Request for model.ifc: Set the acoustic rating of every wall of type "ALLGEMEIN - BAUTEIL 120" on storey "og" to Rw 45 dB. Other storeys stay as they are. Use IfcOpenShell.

First a look at what the model holds.

```python
import ifcopenshell
import ifcopenshell.util.element

model = ifcopenshell.open("model.ifc")
print(model.schema)
storey = next(s for s in model.by_type("IfcBuildingStorey") if s.Name == "og")
walls = [e for e in ifcopenshell.util.element.get_decomposition(storey) if e.is_a("IfcWall")]
seen = {}
for e in walls:
    element_type = ifcopenshell.util.element.get_type(e)
    key = (element_type.Name if element_type != e and element_type else None, ifcopenshell.util.element.get_pset(e, "Pset_WallCommon", "AcousticRating"))
    seen[key] = seen.get(key, 0) + 1
for (name, value), count in sorted(seen.items(), key=str):
    print(count, "x", name, "|", value)
```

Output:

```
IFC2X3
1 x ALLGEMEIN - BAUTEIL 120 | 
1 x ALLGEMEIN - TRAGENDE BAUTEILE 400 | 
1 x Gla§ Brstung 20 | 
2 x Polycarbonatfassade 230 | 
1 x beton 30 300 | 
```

```python
import ifcopenshell
import ifcopenshell.api.pset
import ifcopenshell.util.element

model = ifcopenshell.open("model.ifc")

storey = next(s for s in model.by_type("IfcBuildingStorey") if s.Name == "og")
walls = [e for e in ifcopenshell.util.element.get_decomposition(storey) if e.is_a("IfcWall")]

count = 0
for e in walls:
    element_type = ifcopenshell.util.element.get_type(e)
    if element_type in (None, e) or element_type.Name != "ALLGEMEIN - BAUTEIL 120":
        continue
    # add_pset returns the element's existing set when there is one.
    pset = ifcopenshell.api.pset.add_pset(model, product=e, name="Pset_WallCommon")
    ifcopenshell.api.pset.edit_pset(model, pset=pset, properties={"AcousticRating": "Rw 45 dB"})
    count += 1

print(count, "walls updated")

model.write("model_v2.ifc")
```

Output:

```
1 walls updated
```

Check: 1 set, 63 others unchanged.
